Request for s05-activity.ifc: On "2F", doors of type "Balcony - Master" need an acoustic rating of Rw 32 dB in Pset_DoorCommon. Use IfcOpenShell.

First a look at what the model holds.

```python
import ifcopenshell
import ifcopenshell.util.element

model = ifcopenshell.open("s05-activity.ifc")
print(model.schema)
storey = next(s for s in model.by_type("IfcBuildingStorey") if s.Name == "2F")
doors = [e for e in ifcopenshell.util.element.get_decomposition(storey) if e.is_a("IfcDoor")]
seen = {}
for e in doors:
    element_type = ifcopenshell.util.element.get_type(e)
    key = (element_type.Name if element_type != e and element_type else None, ifcopenshell.util.element.get_pset(e, "Pset_DoorCommon", "AcousticRating"))
    seen[key] = seen.get(key, 0) + 1
for (name, value), count in sorted(seen.items(), key=str):
    print(count, "x", name, "|", value)
```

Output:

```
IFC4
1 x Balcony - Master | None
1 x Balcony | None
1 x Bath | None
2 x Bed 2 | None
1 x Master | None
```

```python
import ifcopenshell
import ifcopenshell.api.pset
import ifcopenshell.util.element

model = ifcopenshell.open("s05-activity.ifc")

storey = next(s for s in model.by_type("IfcBuildingStorey") if s.Name == "2F")
doors = [e for e in ifcopenshell.util.element.get_decomposition(storey) if e.is_a("IfcDoor")]

count = 0
for e in doors:
    element_type = ifcopenshell.util.element.get_type(e)
    if element_type in (None, e) or element_type.Name != "Balcony - Master":
        continue
    # add_pset returns the element's existing set when there is one.
    pset = ifcopenshell.api.pset.add_pset(model, product=e, name="Pset_DoorCommon")
    ifcopenshell.api.pset.edit_pset(model, pset=pset, properties={"AcousticRating": "Rw 32 dB"})
    count += 1

print(count, "doors updated")

model.write("s05-activity_rev.ifc")
```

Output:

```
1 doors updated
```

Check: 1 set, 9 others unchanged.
